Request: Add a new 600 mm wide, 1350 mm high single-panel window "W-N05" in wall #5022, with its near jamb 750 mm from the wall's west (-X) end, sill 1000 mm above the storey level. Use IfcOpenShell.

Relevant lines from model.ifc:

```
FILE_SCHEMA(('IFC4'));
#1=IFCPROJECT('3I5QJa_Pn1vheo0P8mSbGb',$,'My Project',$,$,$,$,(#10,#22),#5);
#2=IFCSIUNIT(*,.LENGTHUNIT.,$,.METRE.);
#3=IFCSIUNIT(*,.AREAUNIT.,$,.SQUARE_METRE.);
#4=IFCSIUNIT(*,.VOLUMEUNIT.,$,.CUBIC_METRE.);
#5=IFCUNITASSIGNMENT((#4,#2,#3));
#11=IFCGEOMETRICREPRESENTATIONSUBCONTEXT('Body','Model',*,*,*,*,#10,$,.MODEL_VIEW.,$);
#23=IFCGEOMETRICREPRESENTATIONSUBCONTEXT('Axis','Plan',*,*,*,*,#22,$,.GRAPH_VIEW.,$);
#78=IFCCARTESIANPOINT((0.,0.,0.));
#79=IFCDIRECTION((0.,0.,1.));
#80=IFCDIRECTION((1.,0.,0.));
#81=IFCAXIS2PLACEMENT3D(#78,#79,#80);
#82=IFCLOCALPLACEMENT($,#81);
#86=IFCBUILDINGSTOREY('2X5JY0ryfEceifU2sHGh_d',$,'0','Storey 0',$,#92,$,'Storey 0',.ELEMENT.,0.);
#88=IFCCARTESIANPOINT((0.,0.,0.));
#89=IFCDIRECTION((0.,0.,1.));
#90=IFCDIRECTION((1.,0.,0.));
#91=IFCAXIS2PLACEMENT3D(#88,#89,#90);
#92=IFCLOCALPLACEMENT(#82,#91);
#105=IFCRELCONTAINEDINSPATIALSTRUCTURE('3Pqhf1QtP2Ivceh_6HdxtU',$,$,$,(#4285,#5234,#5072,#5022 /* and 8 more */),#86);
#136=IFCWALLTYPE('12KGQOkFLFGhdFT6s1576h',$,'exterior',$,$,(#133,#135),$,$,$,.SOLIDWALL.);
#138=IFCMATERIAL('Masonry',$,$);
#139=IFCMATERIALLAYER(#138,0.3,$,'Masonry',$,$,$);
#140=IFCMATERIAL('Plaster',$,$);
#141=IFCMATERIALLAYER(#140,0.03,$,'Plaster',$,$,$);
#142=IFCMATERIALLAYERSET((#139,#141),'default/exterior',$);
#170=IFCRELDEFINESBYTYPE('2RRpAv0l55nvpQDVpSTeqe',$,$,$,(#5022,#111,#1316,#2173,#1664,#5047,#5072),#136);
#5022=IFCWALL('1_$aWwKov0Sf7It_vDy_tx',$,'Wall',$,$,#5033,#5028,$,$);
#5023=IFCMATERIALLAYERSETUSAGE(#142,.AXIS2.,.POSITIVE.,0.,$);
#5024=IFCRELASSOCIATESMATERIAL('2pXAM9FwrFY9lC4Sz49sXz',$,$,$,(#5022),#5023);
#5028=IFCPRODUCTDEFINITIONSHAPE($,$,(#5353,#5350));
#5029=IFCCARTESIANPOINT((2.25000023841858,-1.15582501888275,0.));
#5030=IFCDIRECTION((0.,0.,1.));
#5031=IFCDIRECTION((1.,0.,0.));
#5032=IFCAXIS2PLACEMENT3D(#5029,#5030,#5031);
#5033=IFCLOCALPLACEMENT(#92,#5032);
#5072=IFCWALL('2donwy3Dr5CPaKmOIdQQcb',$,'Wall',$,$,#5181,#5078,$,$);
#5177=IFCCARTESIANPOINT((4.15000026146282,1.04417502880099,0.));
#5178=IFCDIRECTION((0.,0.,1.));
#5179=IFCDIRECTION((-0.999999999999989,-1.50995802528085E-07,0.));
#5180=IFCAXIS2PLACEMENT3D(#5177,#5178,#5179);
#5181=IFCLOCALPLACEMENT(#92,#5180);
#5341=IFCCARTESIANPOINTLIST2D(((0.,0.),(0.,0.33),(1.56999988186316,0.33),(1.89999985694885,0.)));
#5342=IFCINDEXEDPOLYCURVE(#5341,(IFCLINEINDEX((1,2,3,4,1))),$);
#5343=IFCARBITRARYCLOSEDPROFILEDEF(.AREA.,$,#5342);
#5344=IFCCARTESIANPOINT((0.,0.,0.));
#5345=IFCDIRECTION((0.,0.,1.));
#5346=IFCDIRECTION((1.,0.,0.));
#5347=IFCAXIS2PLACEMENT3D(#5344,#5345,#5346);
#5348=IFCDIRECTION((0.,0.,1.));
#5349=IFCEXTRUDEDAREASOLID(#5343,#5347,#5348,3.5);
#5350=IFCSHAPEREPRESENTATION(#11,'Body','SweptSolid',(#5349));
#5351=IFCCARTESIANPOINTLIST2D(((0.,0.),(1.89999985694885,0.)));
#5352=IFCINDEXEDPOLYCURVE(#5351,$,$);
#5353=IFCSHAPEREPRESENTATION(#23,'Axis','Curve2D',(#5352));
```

```python
import numpy as np
import ifcopenshell
import ifcopenshell.api.feature
import ifcopenshell.api.geometry
import ifcopenshell.api.root
import ifcopenshell.api.spatial
import ifcopenshell.geom
import ifcopenshell.util.element
import ifcopenshell.util.placement
import ifcopenshell.util.representation
import ifcopenshell.util.shape
import ifcopenshell.util.unit

model = ifcopenshell.open("model.ifc")
unit_scale = ifcopenshell.util.unit.calculate_unit_scale(model)
settings = ifcopenshell.geom.settings()


def volume(element):
    """Net volume in cubic metres, openings subtracted."""
    shape = ifcopenshell.geom.create_shape(settings, element)
    return ifcopenshell.util.shape.get_volume(shape.geometry)


wall = model.by_guid("1_$aWwKov0Sf7It_vDy_tx")
storey = ifcopenshell.util.element.get_container(wall, ifc_class="IfcBuildingStorey")
context = ifcopenshell.util.representation.get_context(model, "Model", "Body", "MODEL_VIEW")
before = volume(wall)

width, height, from_end, sill = 0.6, 1.35, 0.75, 1  # metres

# The wall runs along its own X axis, and the end named is its -X end.
wall_shape = ifcopenshell.geom.create_shape(settings, wall)
x, y, z = ifcopenshell.util.shape.get_vertices(wall_shape.geometry).T
start = x.min() + from_end
face, thickness = float(y.min()), float(y.max() - y.min())
wall_matrix = ifcopenshell.util.placement.get_local_placement(wall.ObjectPlacement)
level = ifcopenshell.util.placement.get_local_placement(storey.ObjectPlacement)[2, 3]


def in_wall(x, y):
    """Placement at x, y metres in the wall's axes, at sill height."""
    matrix = wall_matrix.copy()
    matrix[:, 3] = wall_matrix @ np.array([x / unit_scale, y / unit_scale, 0.0, 1.0])
    matrix[2, 3] = level + sill / unit_scale
    return matrix


# Opening: a box that overshoots both wall faces by 50 mm.
opening = ifcopenshell.api.root.create_entity(model, ifc_class="IfcOpeningElement", predefined_type="OPENING")
box = ifcopenshell.api.geometry.add_wall_representation(
    model, context=context, length=width, height=height, thickness=thickness + 0.1
)
ifcopenshell.api.geometry.assign_representation(model, product=opening, representation=box)
ifcopenshell.api.geometry.edit_object_placement(model, product=opening, matrix=in_wall(start, face - 0.05), is_si=False)
ifcopenshell.api.feature.add_feature(model, feature=opening, element=wall)

window = ifcopenshell.api.root.create_entity(model, ifc_class="IfcWindow", name="W-N05", predefined_type="WINDOW")
window.OverallWidth, window.OverallHeight = width / unit_scale, height / unit_scale
window.PartitioningType = "SINGLE_PANEL"
body = ifcopenshell.api.geometry.add_window_representation(
    model,
    context=context,
    overall_width=window.OverallWidth,
    overall_height=window.OverallHeight,
    partition_type="SINGLE_PANEL",
)
ifcopenshell.api.geometry.assign_representation(model, product=window, representation=body)
ifcopenshell.api.spatial.assign_container(model, products=[window], relating_structure=storey)
ifcopenshell.api.feature.add_filling(model, opening=opening, element=window)

# Centre the window in the wall's thickness.
ifcopenshell.api.geometry.edit_object_placement(model, product=window, matrix=in_wall(start, face), is_si=False)
window_shape = ifcopenshell.geom.create_shape(settings, window)
depth = ifcopenshell.util.shape.get_vertices(window_shape.geometry)[:, 1]
offset = face + thickness / 2 - (depth.min() + depth.max()) / 2
ifcopenshell.api.geometry.edit_object_placement(model, product=window, matrix=in_wall(start, offset), is_si=False)

after = volume(wall)

print(f"wall volume {before:.3f} -> {after:.3f} m3")

model.write("model_v2.ifc")
```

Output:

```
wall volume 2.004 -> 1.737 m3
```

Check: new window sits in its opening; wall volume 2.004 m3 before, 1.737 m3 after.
